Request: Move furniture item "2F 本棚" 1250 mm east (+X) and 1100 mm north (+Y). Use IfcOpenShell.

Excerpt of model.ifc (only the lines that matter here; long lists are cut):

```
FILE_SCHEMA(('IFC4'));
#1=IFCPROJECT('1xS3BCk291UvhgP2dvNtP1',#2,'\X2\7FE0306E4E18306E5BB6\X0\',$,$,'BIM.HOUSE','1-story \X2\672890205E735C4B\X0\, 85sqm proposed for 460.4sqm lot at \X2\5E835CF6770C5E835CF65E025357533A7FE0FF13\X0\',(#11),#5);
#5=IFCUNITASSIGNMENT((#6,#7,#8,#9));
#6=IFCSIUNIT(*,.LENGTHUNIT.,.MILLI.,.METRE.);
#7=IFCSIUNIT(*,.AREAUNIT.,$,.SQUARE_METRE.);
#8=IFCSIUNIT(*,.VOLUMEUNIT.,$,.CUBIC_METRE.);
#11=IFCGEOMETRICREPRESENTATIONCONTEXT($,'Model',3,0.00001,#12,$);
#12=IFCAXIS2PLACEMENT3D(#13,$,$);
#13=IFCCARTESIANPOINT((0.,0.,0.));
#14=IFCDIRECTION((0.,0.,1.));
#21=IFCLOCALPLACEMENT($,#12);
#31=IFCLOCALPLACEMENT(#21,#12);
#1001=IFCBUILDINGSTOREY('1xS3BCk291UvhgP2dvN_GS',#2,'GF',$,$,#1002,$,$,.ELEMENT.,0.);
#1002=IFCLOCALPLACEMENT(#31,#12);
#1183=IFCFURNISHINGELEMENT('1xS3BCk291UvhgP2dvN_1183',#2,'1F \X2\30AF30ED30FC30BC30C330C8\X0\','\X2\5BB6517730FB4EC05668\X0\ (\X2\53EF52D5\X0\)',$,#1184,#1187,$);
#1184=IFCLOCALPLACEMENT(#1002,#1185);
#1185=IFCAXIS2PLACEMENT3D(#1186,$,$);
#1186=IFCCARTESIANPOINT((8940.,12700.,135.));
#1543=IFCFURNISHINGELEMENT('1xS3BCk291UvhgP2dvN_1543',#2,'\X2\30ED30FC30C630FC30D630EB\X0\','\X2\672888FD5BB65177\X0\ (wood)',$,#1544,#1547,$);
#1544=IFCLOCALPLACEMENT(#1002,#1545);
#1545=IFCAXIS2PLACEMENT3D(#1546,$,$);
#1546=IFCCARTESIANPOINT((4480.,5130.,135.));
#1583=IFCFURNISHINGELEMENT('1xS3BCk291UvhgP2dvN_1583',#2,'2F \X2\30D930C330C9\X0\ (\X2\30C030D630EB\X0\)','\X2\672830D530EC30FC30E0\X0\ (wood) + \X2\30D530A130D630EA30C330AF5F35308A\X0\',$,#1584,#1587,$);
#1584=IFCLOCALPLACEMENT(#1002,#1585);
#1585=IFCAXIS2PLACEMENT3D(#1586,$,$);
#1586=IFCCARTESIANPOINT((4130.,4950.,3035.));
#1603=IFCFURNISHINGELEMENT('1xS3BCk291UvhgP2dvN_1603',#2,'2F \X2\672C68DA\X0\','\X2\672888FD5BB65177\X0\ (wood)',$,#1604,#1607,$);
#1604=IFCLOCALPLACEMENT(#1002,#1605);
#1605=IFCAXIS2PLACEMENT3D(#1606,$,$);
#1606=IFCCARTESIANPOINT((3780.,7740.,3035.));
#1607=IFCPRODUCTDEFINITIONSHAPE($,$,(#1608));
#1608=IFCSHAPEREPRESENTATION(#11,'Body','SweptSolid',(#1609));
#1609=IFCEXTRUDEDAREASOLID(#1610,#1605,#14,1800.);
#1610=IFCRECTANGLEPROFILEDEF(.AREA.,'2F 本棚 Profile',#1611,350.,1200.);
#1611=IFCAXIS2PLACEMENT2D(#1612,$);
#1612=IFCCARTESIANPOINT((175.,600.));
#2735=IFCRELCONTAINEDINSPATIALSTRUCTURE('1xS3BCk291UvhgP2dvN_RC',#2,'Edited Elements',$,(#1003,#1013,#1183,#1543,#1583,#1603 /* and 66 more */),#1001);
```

```python
import ifcopenshell
import ifcopenshell.api.geometry
import ifcopenshell.util.placement
import ifcopenshell.util.unit

model = ifcopenshell.open("model.ifc")
unit_scale = ifcopenshell.util.unit.calculate_unit_scale(model)

item = model.by_id(1603)
matrix = ifcopenshell.util.placement.get_local_placement(item.ObjectPlacement)
matrix[0, 3] += 1.25 / unit_scale
matrix[1, 3] += 1.1 / unit_scale
ifcopenshell.api.geometry.edit_object_placement(model, product=item, matrix=matrix, is_si=False)

print(ifcopenshell.util.placement.get_local_placement(item.ObjectPlacement).round(3) + 0.0)

model.write("model_edited.ifc")
```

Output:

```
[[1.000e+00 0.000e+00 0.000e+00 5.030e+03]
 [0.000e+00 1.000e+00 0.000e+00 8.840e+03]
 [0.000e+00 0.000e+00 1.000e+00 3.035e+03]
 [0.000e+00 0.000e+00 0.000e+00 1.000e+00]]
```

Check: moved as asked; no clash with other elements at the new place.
